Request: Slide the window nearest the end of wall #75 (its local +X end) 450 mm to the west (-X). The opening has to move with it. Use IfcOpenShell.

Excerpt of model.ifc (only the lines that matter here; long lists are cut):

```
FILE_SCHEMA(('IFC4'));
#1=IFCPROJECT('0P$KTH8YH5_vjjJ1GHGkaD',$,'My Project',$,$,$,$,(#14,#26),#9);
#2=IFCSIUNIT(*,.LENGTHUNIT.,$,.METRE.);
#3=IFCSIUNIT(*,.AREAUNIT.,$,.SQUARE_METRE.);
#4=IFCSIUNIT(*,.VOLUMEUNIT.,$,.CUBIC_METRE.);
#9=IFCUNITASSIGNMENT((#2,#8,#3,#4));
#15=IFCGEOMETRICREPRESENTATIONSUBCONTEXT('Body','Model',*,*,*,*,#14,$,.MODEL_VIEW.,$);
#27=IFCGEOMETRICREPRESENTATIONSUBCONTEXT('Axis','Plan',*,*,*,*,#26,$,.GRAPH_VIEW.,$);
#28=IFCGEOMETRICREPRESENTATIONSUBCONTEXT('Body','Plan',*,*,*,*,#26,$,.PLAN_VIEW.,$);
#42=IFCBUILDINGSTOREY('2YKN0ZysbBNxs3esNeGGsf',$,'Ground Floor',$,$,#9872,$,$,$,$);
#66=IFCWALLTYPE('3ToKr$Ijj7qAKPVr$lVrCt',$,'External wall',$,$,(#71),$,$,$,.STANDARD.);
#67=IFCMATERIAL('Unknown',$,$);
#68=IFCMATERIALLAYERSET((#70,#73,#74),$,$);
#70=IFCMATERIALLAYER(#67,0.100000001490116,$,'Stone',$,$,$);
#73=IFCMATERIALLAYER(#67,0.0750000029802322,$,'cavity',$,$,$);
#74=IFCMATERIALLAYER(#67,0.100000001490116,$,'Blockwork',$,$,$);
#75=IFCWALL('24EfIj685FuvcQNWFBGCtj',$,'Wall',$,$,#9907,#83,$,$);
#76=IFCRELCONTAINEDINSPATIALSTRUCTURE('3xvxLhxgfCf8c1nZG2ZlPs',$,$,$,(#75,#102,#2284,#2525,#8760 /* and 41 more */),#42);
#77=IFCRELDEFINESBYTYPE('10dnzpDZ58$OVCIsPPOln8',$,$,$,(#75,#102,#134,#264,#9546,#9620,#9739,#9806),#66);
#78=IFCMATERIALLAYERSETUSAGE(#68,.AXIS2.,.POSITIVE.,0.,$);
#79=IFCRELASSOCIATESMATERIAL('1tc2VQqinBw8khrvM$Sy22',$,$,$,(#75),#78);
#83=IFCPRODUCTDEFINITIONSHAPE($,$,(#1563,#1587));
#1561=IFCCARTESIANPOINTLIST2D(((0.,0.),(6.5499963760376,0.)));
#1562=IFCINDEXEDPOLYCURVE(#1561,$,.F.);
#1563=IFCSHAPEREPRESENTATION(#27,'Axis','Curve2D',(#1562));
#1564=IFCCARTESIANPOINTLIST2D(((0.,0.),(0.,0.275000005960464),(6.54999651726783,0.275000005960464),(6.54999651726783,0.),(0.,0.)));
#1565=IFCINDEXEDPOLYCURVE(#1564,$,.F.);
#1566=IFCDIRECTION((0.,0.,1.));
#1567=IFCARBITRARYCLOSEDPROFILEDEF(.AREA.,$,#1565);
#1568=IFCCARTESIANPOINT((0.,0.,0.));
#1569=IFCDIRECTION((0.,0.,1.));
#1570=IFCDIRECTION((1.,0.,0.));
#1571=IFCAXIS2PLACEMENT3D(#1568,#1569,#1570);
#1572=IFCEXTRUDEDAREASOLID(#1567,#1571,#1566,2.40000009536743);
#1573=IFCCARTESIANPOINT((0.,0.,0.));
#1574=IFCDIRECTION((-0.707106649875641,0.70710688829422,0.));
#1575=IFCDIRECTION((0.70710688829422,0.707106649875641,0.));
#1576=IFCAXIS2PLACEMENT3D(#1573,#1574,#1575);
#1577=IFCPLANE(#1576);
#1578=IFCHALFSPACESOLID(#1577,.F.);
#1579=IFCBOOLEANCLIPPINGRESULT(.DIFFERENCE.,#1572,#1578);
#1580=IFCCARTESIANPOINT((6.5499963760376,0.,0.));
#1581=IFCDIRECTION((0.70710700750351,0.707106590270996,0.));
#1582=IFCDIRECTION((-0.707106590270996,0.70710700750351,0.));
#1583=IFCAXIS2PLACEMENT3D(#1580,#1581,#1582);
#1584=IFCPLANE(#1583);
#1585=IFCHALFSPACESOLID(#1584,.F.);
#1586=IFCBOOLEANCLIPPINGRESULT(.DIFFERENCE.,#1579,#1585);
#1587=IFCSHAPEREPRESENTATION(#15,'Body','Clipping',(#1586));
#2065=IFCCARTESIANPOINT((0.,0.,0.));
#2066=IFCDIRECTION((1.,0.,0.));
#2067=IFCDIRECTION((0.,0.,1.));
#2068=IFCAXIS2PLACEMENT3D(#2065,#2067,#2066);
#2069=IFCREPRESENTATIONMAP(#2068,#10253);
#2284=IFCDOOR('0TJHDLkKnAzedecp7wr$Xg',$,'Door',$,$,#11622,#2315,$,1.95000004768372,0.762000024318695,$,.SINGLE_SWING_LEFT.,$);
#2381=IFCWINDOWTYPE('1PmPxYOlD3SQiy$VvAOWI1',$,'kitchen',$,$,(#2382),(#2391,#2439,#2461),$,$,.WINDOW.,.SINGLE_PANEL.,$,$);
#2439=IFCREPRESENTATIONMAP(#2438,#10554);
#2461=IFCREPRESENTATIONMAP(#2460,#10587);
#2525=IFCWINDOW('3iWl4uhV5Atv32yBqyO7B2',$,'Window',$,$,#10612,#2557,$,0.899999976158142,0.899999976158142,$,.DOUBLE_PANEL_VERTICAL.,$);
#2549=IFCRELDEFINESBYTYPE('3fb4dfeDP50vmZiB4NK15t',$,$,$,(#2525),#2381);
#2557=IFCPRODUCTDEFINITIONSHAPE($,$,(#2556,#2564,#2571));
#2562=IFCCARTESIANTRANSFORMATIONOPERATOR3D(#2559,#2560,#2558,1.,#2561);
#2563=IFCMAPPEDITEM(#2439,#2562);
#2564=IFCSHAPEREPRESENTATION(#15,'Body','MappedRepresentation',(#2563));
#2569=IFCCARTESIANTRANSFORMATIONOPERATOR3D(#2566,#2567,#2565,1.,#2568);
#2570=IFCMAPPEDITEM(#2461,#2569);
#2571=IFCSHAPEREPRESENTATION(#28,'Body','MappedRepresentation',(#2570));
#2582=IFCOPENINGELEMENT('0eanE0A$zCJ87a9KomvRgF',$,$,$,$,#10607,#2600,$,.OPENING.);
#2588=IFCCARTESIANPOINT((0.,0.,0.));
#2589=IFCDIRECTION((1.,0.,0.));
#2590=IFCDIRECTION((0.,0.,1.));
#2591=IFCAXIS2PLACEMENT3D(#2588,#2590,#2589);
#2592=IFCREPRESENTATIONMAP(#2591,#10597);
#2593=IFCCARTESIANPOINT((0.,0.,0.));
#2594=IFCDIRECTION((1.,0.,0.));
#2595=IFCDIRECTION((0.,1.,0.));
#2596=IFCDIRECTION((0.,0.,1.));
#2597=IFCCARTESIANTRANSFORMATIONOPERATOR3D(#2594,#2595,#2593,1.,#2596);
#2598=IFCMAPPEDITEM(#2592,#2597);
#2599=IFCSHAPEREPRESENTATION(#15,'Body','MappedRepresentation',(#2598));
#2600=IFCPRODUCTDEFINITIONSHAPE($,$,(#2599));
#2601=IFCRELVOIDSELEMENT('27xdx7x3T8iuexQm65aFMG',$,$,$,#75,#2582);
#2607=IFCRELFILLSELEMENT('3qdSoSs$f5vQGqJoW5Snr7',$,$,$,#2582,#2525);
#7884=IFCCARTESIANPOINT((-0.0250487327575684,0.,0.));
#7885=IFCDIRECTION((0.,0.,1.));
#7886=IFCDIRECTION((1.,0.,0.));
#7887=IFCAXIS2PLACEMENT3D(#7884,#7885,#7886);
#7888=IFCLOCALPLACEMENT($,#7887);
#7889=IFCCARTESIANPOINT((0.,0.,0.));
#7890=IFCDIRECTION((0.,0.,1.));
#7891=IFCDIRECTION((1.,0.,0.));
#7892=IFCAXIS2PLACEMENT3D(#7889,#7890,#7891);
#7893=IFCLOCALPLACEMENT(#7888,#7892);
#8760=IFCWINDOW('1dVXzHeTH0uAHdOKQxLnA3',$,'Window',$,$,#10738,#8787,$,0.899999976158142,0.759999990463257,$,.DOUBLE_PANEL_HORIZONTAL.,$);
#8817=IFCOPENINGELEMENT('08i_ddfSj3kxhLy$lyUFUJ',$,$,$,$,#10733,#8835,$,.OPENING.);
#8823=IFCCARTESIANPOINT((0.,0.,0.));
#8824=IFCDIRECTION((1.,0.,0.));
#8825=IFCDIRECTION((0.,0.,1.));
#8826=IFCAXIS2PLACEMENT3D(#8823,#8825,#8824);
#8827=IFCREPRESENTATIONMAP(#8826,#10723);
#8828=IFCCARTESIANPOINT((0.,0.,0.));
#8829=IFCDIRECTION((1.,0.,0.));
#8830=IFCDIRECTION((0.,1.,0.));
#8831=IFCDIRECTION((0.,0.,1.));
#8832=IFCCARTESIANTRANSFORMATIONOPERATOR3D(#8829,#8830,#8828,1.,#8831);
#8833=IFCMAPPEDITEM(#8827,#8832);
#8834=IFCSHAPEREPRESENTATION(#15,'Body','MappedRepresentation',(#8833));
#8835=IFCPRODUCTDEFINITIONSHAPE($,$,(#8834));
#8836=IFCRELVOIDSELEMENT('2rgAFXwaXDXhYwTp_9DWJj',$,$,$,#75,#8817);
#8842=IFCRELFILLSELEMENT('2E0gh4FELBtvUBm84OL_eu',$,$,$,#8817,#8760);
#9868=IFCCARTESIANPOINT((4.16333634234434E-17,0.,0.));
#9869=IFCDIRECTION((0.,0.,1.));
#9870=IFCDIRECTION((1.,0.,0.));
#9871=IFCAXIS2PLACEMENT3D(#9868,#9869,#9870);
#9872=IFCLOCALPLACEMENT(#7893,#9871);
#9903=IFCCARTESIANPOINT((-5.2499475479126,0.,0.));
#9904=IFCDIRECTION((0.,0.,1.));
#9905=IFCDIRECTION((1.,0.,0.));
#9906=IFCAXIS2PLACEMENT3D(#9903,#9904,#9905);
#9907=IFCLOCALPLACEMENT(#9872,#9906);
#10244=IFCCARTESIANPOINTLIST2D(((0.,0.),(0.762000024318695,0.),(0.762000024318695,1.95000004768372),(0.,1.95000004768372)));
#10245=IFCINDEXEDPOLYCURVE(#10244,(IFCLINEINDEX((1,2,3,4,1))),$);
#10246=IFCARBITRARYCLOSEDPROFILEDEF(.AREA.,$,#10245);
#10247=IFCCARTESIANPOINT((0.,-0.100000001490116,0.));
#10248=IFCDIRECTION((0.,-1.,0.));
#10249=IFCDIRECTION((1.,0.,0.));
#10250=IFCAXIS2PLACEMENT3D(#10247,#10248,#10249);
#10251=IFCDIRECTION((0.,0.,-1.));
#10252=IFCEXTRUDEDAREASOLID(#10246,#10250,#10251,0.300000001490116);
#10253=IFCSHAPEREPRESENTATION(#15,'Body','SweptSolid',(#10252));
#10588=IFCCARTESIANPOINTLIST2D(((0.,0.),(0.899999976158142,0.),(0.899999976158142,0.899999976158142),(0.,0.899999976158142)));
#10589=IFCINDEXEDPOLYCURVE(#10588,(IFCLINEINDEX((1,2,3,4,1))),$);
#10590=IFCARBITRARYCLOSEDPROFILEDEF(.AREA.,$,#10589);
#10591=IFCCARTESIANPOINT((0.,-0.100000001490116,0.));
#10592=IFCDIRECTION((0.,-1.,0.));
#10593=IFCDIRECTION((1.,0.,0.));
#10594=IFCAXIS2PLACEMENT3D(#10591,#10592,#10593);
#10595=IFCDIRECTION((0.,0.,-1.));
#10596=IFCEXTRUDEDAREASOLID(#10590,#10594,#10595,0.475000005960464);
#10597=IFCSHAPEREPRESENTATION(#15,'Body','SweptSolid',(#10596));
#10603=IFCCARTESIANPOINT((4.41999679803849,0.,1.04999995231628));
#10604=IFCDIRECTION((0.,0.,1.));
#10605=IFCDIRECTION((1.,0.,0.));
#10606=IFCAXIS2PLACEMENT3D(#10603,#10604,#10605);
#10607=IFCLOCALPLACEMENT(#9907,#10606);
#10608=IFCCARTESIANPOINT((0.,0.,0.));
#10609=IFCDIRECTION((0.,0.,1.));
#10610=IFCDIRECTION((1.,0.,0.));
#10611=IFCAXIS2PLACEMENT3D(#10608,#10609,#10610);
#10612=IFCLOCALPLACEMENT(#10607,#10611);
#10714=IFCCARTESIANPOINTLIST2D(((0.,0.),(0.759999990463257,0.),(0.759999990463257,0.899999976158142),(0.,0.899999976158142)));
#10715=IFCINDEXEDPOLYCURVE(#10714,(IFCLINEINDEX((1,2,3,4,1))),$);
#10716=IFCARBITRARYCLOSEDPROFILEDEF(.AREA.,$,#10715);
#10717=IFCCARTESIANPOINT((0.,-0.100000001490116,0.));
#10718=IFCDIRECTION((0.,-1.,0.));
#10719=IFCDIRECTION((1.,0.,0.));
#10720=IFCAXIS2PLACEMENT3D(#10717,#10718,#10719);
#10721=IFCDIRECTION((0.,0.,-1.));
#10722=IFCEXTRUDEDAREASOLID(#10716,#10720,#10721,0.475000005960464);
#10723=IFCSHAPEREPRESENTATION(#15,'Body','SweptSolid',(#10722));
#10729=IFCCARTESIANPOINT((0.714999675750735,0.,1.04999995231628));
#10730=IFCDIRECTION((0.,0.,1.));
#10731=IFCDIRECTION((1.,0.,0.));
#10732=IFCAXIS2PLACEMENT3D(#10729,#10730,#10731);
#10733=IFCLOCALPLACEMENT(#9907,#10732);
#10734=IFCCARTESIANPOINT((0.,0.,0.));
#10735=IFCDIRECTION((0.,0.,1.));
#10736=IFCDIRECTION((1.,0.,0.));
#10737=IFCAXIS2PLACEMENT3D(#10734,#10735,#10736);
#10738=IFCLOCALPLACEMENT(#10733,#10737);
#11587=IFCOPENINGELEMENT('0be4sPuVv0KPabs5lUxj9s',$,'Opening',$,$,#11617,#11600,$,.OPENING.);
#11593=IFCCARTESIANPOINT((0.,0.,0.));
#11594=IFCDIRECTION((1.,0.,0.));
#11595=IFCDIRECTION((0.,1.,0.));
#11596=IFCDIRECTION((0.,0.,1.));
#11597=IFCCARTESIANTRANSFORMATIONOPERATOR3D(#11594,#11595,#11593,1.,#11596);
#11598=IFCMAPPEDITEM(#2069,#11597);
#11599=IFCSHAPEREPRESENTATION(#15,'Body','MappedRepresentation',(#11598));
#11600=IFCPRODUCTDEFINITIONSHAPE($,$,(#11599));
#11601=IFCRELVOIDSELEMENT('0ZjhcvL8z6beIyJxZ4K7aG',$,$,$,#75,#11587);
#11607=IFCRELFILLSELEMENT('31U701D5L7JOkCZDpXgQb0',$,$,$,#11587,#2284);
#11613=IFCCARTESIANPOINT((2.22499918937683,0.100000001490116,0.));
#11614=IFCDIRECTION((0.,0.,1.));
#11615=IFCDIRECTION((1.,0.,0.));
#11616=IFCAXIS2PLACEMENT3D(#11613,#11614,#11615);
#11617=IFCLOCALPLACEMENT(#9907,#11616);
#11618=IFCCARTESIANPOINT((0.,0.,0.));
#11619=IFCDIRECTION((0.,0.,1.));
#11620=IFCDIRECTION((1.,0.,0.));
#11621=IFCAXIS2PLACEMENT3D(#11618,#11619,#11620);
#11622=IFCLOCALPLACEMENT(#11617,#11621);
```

```python
import ifcopenshell
import ifcopenshell.api.geometry
import ifcopenshell.util.placement

model = ifcopenshell.open("model.ifc")

window = model.by_id(2525)
opening = window.FillsVoids[0].RelatingOpeningElement
wall = opening.VoidsElements[0].RelatingBuildingElement

wall_matrix = ifcopenshell.util.placement.get_local_placement(wall.ObjectPlacement)
shift = wall_matrix[:3, 0] * -0.45
before = ifcopenshell.util.placement.get_local_placement(window.ObjectPlacement)[:3, 3].copy()

# The window is placed relative to its opening, so it follows when the opening moves.
matrix = ifcopenshell.util.placement.get_local_placement(opening.ObjectPlacement)
matrix[:3, 3] += shift
ifcopenshell.api.geometry.edit_object_placement(
    model, product=opening, matrix=matrix, is_si=False, should_transform_children=True
)

after = ifcopenshell.util.placement.get_local_placement(window.ObjectPlacement)[:3, 3]
print("window moved by", (after - before).round(3) + 0.0)

model.write("model_v2.ifc")
```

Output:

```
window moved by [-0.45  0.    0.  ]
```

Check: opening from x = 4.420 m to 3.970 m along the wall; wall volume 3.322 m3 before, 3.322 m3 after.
